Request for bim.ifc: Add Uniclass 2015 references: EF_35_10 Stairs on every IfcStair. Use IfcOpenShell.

First a look at what the model holds.

```python
import ifcopenshell

model = ifcopenshell.open("bim.ifc")
print(model.schema)
print("classifications:", [c.Name for c in model.by_type("IfcClassification")])
for ifc_class in ("IfcDoor", "IfcRoof", "IfcStair", "IfcWall", "IfcWindow"):
    print(ifc_class, len(model.by_type(ifc_class)))
```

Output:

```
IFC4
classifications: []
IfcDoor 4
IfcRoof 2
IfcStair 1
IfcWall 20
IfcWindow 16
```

```python
import ifcopenshell
import ifcopenshell.api.classification

model = ifcopenshell.open("bim.ifc")

system = ifcopenshell.api.classification.add_classification(model, classification="Uniclass 2015")

codes = {
    "IfcStair": ("EF_35_10", "Stairs"),
}
for ifc_class, (code, name) in codes.items():
    products = model.by_type(ifc_class)
    ifcopenshell.api.classification.add_reference(
        model, products=products, classification=system, identification=code, name=name
    )
    print(code, len(products))

model.write("bim_updated.ifc")
```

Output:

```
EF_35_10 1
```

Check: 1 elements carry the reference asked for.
